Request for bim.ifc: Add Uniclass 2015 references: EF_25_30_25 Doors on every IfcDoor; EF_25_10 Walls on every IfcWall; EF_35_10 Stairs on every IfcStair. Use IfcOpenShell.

First a look at what the model holds.

```python
import ifcopenshell

model = ifcopenshell.open("bim.ifc")
print(model.schema)
print("classifications:", [c.Name for c in model.by_type("IfcClassification")])
for ifc_class in ("IfcDoor", "IfcRoof", "IfcStair", "IfcWall", "IfcWindow"):
    print(ifc_class, len(model.by_type(ifc_class)))
```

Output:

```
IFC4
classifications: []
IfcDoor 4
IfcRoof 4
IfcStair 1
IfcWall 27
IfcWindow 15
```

```python
import ifcopenshell
import ifcopenshell.api.classification

model = ifcopenshell.open("bim.ifc")

system = ifcopenshell.api.classification.add_classification(model, classification="Uniclass 2015")

codes = {
    "IfcDoor": ("EF_25_30_25", "Doors"),
    "IfcWall": ("EF_25_10", "Walls"),
    "IfcStair": ("EF_35_10", "Stairs"),
}
for ifc_class, (code, name) in codes.items():
    products = model.by_type(ifc_class)
    ifcopenshell.api.classification.add_reference(
        model, products=products, classification=system, identification=code, name=name
    )
    print(code, len(products))

model.write("bim_edited.ifc")
```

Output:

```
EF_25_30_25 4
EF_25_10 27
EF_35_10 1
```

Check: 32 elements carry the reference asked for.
